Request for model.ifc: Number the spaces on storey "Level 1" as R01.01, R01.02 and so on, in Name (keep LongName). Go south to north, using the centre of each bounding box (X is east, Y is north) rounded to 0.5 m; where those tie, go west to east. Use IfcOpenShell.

First a look at what the model holds.

```python
import ifcopenshell
import ifcopenshell.util.element
import ifcopenshell.util.placement

model = ifcopenshell.open("model.ifc")
print(model.schema)
storey = next(s for s in model.by_type("IfcBuildingStorey") if s.Name == "Level 1")
spaces = [e for e in ifcopenshell.util.element.get_decomposition(storey) if e.is_a("IfcSpace")]
for e in sorted(spaces, key=lambda e: e.id()):
    origin = ifcopenshell.util.placement.get_local_placement(e.ObjectPlacement)[:3, 3]
    print(e.id(), e.Name, e.LongName, origin.round(2) + 0.0, sep=" | ")
```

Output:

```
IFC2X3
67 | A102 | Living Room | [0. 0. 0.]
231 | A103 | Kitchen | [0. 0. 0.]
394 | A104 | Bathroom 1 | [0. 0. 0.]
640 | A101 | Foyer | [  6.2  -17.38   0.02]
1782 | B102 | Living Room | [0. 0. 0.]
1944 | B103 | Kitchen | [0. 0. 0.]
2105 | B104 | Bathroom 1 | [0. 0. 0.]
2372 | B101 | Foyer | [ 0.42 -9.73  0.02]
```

```python
import ifcopenshell
import ifcopenshell.geom
import ifcopenshell.util.element
import ifcopenshell.util.shape

model = ifcopenshell.open("model.ifc")
settings = ifcopenshell.geom.settings()
settings.set("use-world-coords", True)


def centre(element):
    shape = ifcopenshell.geom.create_shape(settings, element)
    return ifcopenshell.util.shape.get_bbox_centroid(shape.geometry)


storey = next(s for s in model.by_type("IfcBuildingStorey") if s.Name == "Level 1")
spaces = [e for e in ifcopenshell.util.element.get_decomposition(storey) if e.is_a("IfcSpace")]

# Insertion points can sit at a corner or the storey origin, so sort by the geometry (in metres).
centres = {e: centre(e) for e in spaces}
spaces.sort(key=lambda e: (round(centres[e][1] / 0.5), centres[e][0]))

for i, e in enumerate(spaces, start=1):
    number = f"R01.{i:02d}"
    e.Name = number
    print(e.id(), number)

model.write("model_v2.ifc")
```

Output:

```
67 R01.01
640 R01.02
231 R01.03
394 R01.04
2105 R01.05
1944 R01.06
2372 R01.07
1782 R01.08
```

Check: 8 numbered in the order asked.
